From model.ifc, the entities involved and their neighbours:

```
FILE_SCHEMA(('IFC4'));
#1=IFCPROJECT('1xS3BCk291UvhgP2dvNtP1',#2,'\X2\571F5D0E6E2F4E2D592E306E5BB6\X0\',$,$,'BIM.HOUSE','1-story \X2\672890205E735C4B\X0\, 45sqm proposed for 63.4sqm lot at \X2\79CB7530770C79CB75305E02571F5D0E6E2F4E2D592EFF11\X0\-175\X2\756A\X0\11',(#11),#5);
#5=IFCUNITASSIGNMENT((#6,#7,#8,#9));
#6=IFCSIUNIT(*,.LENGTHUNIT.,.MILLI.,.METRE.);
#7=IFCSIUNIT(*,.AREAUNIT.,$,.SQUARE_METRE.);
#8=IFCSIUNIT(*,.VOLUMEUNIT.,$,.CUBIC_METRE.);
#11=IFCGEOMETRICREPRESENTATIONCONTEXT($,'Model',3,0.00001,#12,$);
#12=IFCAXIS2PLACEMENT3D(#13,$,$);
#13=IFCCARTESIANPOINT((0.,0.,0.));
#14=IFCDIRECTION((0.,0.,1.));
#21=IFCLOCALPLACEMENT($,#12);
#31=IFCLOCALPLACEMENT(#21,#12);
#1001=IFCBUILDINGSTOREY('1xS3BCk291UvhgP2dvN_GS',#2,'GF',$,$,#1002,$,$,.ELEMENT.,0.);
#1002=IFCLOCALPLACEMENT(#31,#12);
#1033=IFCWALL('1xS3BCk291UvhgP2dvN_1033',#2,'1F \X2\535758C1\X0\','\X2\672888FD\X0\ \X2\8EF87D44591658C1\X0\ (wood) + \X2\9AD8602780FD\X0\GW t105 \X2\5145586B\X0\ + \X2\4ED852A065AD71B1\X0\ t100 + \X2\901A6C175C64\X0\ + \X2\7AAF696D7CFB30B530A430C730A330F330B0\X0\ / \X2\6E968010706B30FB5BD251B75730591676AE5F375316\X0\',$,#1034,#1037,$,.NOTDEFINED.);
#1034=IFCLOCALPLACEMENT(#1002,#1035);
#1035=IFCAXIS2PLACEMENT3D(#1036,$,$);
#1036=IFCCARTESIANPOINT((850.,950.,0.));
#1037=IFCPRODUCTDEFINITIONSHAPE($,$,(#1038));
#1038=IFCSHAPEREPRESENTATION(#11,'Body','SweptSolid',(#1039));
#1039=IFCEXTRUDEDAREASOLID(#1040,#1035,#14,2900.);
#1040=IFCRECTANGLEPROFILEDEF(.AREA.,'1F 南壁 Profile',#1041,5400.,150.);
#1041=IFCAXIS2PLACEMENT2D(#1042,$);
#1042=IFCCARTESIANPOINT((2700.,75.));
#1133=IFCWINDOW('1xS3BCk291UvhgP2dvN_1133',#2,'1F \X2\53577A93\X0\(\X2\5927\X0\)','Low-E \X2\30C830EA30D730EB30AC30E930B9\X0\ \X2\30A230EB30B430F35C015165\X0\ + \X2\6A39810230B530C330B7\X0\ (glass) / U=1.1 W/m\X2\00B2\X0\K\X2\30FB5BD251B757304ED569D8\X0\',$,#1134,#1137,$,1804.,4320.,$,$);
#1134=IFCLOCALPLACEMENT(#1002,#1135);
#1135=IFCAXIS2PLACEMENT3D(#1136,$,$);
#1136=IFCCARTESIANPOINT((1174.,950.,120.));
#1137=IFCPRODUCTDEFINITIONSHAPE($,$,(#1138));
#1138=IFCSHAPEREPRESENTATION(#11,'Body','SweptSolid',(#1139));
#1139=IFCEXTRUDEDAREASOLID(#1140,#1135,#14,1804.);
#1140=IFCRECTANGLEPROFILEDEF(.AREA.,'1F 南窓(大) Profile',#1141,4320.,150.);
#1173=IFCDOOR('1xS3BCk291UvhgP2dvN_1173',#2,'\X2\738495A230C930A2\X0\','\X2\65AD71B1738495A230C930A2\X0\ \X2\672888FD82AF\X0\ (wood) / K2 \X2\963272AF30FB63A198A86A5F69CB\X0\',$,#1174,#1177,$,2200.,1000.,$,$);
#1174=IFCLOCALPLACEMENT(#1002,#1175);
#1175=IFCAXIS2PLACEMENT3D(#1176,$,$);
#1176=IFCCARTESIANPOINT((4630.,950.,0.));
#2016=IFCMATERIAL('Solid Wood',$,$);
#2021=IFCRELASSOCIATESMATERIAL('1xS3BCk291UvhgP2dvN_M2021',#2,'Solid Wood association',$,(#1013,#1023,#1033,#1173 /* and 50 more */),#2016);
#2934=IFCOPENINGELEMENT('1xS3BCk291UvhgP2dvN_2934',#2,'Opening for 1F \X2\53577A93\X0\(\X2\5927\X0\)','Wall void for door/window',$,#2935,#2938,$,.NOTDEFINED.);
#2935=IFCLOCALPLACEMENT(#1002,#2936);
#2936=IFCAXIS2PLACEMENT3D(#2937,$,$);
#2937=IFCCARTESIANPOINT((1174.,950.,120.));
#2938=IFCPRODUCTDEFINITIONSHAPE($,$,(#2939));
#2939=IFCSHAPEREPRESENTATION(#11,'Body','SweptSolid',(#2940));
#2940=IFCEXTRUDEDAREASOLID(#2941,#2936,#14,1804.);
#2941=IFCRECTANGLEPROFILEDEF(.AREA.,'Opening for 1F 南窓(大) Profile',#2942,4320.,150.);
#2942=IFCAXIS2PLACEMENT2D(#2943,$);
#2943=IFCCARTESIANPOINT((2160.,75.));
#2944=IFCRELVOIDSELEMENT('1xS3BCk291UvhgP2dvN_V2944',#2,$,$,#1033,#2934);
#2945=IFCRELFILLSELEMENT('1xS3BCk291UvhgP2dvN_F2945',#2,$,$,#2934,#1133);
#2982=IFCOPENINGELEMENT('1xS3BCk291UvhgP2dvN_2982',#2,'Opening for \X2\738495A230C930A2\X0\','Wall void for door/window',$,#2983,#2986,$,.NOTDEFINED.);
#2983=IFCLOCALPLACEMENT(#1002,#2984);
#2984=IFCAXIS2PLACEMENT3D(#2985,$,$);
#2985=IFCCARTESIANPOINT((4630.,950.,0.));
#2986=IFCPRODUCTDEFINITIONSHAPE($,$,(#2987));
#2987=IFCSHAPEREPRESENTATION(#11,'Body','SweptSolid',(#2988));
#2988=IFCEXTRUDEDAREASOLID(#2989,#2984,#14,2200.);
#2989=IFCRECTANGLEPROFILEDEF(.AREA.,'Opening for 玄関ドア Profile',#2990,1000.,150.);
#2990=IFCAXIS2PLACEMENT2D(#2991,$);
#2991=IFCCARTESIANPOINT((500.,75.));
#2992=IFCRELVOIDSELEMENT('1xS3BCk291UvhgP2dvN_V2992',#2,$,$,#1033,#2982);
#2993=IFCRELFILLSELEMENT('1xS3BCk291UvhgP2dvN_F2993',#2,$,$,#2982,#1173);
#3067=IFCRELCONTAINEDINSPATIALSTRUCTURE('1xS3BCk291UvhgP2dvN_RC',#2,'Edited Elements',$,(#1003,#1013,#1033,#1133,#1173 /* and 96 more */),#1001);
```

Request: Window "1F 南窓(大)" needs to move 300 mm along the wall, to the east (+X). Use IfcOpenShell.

```python
import ifcopenshell
import ifcopenshell.api.geometry
import ifcopenshell.util.placement
import ifcopenshell.util.unit

model = ifcopenshell.open("model.ifc")
unit_scale = ifcopenshell.util.unit.calculate_unit_scale(model)

window = model.by_id(1133)
opening = window.FillsVoids[0].RelatingOpeningElement
wall = opening.VoidsElements[0].RelatingBuildingElement

wall_matrix = ifcopenshell.util.placement.get_local_placement(wall.ObjectPlacement)
shift = wall_matrix[:3, 0] * 0.3 / unit_scale
before = ifcopenshell.util.placement.get_local_placement(window.ObjectPlacement)[:3, 3].copy()

# The window is not placed relative to its opening, so move both.
for product in (opening, window):
    matrix = ifcopenshell.util.placement.get_local_placement(product.ObjectPlacement)
    matrix[:3, 3] += shift
    ifcopenshell.api.geometry.edit_object_placement(model, product=product, matrix=matrix, is_si=False)

after = ifcopenshell.util.placement.get_local_placement(window.ObjectPlacement)[:3, 3]
print("window moved by", (after - before).round(3) + 0.0)

model.write("model_rev.ifc")
```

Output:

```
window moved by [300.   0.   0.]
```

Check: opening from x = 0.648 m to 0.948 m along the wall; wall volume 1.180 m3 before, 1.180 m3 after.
